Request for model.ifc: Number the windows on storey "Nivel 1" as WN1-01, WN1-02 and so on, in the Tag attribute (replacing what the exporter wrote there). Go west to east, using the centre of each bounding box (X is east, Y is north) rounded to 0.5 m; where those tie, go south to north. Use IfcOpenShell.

First a look at what the model holds.

```python
import ifcopenshell
import ifcopenshell.util.element
import ifcopenshell.util.placement

model = ifcopenshell.open("model.ifc")
print(model.schema)
storey = next(s for s in model.by_type("IfcBuildingStorey") if s.Name == "Nivel 1")
windows = [e for e in ifcopenshell.util.element.get_decomposition(storey) if e.is_a("IfcWindow")]
for e in sorted(windows, key=lambda e: e.id()):
    origin = ifcopenshell.util.placement.get_local_placement(e.ObjectPlacement)[:3, 3]
    print(e.id(), e.Tag, e.Name, origin.round(2) + 0.0, sep=" | ")
```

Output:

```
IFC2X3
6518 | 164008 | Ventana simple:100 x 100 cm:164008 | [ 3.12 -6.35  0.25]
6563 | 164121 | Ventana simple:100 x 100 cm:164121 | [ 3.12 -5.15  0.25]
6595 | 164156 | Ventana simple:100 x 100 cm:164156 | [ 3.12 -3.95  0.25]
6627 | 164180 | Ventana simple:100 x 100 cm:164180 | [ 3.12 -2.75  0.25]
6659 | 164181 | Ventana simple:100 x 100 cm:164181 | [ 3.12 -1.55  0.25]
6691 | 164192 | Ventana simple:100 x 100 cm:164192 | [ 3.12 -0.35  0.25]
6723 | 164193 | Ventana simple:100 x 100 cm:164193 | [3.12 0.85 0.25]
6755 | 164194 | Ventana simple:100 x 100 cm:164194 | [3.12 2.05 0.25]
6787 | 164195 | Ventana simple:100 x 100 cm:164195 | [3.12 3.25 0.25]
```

```python
import ifcopenshell
import ifcopenshell.geom
import ifcopenshell.util.element
import ifcopenshell.util.shape

model = ifcopenshell.open("model.ifc")
settings = ifcopenshell.geom.settings()
settings.set("use-world-coords", True)


def centre(element):
    shape = ifcopenshell.geom.create_shape(settings, element)
    return ifcopenshell.util.shape.get_bbox_centroid(shape.geometry)


storey = next(s for s in model.by_type("IfcBuildingStorey") if s.Name == "Nivel 1")
windows = [e for e in ifcopenshell.util.element.get_decomposition(storey) if e.is_a("IfcWindow")]

# Insertion points can sit at a corner or the storey origin, so sort by the geometry (in metres).
centres = {e: centre(e) for e in windows}
windows.sort(key=lambda e: (round(centres[e][0] / 0.5), centres[e][1]))

for i, e in enumerate(windows, start=1):
    number = f"WN1-{i:02d}"
    e.Tag = number
    print(e.id(), number)

model.write("model_edited.ifc")
```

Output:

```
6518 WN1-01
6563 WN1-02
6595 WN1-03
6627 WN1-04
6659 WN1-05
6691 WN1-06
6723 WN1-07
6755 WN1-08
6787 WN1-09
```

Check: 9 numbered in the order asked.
